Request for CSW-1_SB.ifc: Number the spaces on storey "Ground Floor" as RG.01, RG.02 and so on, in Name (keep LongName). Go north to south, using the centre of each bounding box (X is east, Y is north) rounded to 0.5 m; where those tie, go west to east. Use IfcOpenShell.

First a look at what the model holds.

```python
import ifcopenshell
import ifcopenshell.util.element
import ifcopenshell.util.placement

model = ifcopenshell.open("CSW-1_SB.ifc")
print(model.schema)
storey = next(s for s in model.by_type("IfcBuildingStorey") if s.Name == "Ground Floor")
spaces = [e for e in ifcopenshell.util.element.get_decomposition(storey) if e.is_a("IfcSpace")]
for e in sorted(spaces, key=lambda e: e.id()):
    origin = ifcopenshell.util.placement.get_local_placement(e.ObjectPlacement)[:3, 3]
    print(e.id(), e.Name, e.LongName, origin.round(2) + 0.0, sep=" | ")
```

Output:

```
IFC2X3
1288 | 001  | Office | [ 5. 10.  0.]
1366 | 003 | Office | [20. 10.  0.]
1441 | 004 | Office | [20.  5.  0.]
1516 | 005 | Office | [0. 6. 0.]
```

```python
import ifcopenshell
import ifcopenshell.geom
import ifcopenshell.util.element
import ifcopenshell.util.shape

model = ifcopenshell.open("CSW-1_SB.ifc")
settings = ifcopenshell.geom.settings()
settings.set("use-world-coords", True)


def centre(element):
    shape = ifcopenshell.geom.create_shape(settings, element)
    return ifcopenshell.util.shape.get_bbox_centroid(shape.geometry)


storey = next(s for s in model.by_type("IfcBuildingStorey") if s.Name == "Ground Floor")
spaces = [e for e in ifcopenshell.util.element.get_decomposition(storey) if e.is_a("IfcSpace")]

# Insertion points can sit at a corner or the storey origin, so sort by the geometry (in metres).
centres = {e: centre(e) for e in spaces}
spaces.sort(key=lambda e: (-round(centres[e][1] / 0.5), centres[e][0]))

for i, e in enumerate(spaces, start=1):
    number = f"RG.{i:02d}"
    e.Name = number
    print(e.id(), number)

model.write("CSW-1_SB_edited.ifc")
```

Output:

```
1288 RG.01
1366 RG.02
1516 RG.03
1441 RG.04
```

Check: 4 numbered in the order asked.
